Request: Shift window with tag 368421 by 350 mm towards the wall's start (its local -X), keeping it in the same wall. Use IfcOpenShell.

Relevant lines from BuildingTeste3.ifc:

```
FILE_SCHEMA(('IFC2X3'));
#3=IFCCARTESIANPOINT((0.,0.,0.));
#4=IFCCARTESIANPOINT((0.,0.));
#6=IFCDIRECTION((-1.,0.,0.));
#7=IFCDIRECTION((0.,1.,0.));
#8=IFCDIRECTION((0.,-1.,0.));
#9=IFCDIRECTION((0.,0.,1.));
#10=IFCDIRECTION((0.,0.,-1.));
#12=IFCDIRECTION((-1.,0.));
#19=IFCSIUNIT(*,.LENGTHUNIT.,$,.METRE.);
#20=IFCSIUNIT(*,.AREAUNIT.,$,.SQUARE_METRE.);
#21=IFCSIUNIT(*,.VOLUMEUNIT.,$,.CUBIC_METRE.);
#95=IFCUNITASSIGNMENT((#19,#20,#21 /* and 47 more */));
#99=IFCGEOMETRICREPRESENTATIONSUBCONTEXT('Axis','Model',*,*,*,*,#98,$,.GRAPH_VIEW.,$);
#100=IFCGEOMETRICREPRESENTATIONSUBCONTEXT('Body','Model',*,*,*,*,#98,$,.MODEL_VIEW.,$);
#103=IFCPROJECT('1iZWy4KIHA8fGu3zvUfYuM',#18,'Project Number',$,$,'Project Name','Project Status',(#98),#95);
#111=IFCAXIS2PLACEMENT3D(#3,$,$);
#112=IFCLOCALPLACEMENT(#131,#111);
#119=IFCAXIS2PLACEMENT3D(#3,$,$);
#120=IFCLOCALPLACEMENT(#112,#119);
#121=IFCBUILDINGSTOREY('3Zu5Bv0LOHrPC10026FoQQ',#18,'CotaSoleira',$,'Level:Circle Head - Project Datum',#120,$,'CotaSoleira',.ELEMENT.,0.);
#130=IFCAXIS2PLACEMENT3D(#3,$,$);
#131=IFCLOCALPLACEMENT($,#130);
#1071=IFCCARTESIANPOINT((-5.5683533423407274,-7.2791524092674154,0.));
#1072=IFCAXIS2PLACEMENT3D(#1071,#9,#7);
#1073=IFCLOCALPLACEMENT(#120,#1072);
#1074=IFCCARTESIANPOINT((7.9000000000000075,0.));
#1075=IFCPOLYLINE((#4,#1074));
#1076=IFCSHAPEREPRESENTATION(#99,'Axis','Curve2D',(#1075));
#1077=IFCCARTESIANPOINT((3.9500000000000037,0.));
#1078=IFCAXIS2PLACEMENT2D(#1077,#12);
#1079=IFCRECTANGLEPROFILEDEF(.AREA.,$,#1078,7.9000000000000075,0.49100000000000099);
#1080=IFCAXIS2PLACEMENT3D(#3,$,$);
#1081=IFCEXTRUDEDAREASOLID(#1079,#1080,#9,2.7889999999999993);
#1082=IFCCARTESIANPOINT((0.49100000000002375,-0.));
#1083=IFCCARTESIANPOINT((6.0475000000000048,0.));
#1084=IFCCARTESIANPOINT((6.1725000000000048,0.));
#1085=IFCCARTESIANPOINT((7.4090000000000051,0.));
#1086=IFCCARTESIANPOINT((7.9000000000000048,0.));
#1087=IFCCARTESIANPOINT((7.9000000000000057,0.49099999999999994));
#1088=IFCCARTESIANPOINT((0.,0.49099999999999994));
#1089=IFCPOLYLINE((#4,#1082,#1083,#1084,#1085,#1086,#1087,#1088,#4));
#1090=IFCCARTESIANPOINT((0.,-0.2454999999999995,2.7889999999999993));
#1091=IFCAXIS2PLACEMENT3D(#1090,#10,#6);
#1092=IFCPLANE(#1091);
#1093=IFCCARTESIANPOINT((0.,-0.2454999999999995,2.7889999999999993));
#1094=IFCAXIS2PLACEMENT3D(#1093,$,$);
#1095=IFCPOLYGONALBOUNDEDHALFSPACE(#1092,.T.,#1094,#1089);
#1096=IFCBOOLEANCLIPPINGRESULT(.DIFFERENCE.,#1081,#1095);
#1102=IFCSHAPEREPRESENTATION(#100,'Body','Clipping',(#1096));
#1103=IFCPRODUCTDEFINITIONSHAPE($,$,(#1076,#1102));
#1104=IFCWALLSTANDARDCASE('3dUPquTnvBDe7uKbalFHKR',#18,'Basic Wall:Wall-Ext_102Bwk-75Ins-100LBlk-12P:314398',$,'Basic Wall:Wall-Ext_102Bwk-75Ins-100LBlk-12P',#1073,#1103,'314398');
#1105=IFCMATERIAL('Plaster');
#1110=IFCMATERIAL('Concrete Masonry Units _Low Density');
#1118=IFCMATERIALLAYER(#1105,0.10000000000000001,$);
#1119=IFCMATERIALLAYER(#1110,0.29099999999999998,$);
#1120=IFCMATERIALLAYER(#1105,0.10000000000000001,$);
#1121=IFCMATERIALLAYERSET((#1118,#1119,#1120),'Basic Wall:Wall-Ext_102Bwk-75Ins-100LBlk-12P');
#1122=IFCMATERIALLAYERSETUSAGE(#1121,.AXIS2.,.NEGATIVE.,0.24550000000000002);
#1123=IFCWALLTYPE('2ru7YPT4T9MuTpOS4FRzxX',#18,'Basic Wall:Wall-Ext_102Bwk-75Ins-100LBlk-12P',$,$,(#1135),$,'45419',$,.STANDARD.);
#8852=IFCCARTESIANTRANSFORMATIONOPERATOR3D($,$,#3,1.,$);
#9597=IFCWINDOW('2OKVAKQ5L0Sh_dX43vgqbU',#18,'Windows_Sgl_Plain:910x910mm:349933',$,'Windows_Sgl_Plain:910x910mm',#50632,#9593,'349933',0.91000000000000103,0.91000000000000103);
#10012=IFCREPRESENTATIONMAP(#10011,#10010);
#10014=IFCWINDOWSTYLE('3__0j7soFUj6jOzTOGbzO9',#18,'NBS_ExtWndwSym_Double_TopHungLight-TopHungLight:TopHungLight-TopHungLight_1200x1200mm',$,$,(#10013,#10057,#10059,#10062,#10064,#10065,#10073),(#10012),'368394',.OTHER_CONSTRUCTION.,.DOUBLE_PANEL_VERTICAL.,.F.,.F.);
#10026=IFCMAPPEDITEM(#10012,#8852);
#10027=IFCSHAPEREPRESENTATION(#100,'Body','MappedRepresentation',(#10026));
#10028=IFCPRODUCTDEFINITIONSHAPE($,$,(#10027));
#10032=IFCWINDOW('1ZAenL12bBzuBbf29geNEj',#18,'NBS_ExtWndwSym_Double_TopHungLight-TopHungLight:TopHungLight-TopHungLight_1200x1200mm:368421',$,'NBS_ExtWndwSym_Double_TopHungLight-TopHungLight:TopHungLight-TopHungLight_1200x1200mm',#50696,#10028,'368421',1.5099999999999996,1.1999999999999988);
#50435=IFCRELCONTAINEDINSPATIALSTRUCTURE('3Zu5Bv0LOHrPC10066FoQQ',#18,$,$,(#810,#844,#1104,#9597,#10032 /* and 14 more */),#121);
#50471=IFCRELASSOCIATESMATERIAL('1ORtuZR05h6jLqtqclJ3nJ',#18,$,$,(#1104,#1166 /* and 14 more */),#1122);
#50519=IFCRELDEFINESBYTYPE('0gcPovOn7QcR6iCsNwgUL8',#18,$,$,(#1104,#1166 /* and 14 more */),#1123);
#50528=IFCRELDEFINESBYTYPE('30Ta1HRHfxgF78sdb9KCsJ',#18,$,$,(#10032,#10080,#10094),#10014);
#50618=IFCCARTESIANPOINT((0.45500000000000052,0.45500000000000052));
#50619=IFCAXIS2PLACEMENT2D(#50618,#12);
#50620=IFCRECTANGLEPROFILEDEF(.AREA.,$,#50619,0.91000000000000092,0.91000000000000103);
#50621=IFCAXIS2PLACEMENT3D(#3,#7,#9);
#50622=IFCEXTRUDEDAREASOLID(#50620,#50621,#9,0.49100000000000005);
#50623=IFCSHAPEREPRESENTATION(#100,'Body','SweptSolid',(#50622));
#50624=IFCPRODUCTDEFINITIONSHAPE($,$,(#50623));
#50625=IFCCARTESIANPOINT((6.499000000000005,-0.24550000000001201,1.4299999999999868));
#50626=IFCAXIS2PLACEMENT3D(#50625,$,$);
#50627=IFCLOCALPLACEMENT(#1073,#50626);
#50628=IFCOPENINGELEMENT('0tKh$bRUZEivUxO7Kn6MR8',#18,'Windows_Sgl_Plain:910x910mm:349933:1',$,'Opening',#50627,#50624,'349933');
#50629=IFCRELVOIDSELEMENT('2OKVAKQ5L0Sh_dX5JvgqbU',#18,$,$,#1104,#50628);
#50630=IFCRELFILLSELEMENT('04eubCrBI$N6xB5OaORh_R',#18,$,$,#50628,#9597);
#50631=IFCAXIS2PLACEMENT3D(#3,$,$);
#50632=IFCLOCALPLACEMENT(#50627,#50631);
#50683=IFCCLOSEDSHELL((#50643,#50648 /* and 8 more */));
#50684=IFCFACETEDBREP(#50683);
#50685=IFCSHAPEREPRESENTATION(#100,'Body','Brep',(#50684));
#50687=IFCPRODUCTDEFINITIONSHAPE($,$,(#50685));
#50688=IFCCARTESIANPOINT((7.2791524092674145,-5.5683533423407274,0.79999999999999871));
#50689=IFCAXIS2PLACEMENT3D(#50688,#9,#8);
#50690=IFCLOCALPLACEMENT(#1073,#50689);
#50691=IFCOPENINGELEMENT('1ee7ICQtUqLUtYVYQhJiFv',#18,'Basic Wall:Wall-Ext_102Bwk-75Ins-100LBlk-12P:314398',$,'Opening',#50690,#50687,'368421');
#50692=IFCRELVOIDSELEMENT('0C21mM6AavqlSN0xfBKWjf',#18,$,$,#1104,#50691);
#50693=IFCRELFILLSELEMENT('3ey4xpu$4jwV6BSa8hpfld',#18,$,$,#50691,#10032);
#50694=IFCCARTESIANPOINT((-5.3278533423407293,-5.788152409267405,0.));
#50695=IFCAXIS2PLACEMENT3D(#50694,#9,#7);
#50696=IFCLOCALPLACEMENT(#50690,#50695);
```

```python
import ifcopenshell
import ifcopenshell.api.geometry
import ifcopenshell.util.placement
import ifcopenshell.util.unit

model = ifcopenshell.open("BuildingTeste3.ifc")
unit_scale = ifcopenshell.util.unit.calculate_unit_scale(model)

window = model.by_guid("1ZAenL12bBzuBbf29geNEj")
opening = window.FillsVoids[0].RelatingOpeningElement
wall = opening.VoidsElements[0].RelatingBuildingElement

wall_matrix = ifcopenshell.util.placement.get_local_placement(wall.ObjectPlacement)
shift = wall_matrix[:3, 0] * -0.35 / unit_scale
before = ifcopenshell.util.placement.get_local_placement(window.ObjectPlacement)[:3, 3].copy()

# The window is placed relative to its opening, so it follows when the opening moves.
matrix = ifcopenshell.util.placement.get_local_placement(opening.ObjectPlacement)
matrix[:3, 3] += shift
ifcopenshell.api.geometry.edit_object_placement(
    model, product=opening, matrix=matrix, is_si=False, should_transform_children=True
)

after = ifcopenshell.util.placement.get_local_placement(window.ObjectPlacement)[:3, 3]
print("window moved by", (after - before).round(3) + 0.0)

model.write("BuildingTeste3_rev.ifc")
```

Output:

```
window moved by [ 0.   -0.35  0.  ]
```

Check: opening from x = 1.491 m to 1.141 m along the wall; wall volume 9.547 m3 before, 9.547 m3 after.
